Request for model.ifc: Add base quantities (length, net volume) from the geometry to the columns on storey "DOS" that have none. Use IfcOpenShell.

First a look at what the model holds.

```python
import ifcopenshell
import ifcopenshell.util.element
import ifcopenshell.util.unit

model = ifcopenshell.open("model.ifc")
print(model.schema)
for unit_type in ("LENGTHUNIT", "AREAUNIT", "VOLUMEUNIT"):
    print(unit_type, ifcopenshell.util.unit.calculate_unit_scale(model, unit_type))
storey = next(s for s in model.by_type("IfcBuildingStorey") if s.Name == "DOS")
columns = [e for e in ifcopenshell.util.element.get_decomposition(storey) if e.is_a("IfcColumn")]
for e in sorted(columns, key=lambda e: e.id()):
    print(e.id(), e.is_a(), e.Name, list(ifcopenshell.util.element.get_psets(e, qtos_only=True)), sep=" | ")
```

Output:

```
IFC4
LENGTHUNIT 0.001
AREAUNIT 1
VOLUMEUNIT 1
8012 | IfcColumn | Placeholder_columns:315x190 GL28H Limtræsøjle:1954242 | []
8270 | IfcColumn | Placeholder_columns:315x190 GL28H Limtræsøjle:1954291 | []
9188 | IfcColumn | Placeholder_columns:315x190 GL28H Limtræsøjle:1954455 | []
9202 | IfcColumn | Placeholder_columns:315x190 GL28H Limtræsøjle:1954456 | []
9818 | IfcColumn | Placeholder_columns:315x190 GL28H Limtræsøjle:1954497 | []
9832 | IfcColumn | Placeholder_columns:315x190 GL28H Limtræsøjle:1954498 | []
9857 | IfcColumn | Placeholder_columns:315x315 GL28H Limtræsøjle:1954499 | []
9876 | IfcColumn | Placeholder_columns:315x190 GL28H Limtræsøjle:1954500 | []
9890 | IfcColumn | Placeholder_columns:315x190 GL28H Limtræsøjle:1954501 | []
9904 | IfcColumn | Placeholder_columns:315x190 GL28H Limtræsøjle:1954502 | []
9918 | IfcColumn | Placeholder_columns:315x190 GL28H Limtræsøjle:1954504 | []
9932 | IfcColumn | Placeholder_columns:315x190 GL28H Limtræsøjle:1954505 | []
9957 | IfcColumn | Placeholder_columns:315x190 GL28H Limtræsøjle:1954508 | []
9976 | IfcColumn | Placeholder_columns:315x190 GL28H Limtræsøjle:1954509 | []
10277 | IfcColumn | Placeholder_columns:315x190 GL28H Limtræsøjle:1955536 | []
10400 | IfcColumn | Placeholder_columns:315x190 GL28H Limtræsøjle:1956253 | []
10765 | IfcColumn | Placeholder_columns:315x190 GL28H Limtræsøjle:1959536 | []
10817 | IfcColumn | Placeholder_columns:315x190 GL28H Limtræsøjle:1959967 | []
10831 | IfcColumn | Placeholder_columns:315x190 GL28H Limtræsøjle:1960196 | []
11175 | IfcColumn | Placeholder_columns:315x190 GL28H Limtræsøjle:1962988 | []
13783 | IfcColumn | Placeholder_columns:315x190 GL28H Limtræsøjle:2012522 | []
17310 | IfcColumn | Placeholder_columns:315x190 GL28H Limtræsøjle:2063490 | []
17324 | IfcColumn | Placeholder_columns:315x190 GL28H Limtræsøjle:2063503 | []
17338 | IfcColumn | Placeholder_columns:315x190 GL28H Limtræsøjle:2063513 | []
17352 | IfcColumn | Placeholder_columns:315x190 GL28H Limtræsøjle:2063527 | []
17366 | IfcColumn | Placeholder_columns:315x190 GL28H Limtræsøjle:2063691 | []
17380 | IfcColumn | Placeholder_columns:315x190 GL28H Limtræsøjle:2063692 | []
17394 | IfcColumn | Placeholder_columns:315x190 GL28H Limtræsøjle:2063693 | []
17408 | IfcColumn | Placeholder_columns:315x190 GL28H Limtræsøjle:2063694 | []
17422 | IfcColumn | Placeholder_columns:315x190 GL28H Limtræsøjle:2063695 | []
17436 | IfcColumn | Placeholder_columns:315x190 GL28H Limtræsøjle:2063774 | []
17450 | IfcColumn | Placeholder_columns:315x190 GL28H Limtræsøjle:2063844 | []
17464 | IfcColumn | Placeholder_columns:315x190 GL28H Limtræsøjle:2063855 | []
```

```python
import ifcopenshell
import ifcopenshell.api.pset
import ifcopenshell.geom
import ifcopenshell.util.element
import ifcopenshell.util.shape
import ifcopenshell.util.unit

model = ifcopenshell.open("model.ifc")
unit_scale = ifcopenshell.util.unit.calculate_unit_scale(model)
volume_scale = ifcopenshell.util.unit.calculate_unit_scale(model, "VOLUMEUNIT")
settings = ifcopenshell.geom.settings()

storey = next(s for s in model.by_type("IfcBuildingStorey") if s.Name == "DOS")
columns = [e for e in ifcopenshell.util.element.get_decomposition(storey) if e.is_a("IfcColumn")]

for e in sorted(columns, key=lambda e: e.id()):
    if ifcopenshell.util.element.get_psets(e, qtos_only=True, should_inherit=False):
        continue
    # Geometry comes back in metres, in the element's own axes.
    shape = ifcopenshell.geom.create_shape(settings, e)
    values = {
        "Length": ifcopenshell.util.shape.get_z(shape.geometry) / unit_scale,
        "NetVolume": ifcopenshell.util.shape.get_volume(shape.geometry) / volume_scale,
    }
    qto = ifcopenshell.api.pset.add_qto(model, product=e, name="Qto_ColumnBaseQuantities")
    ifcopenshell.api.pset.edit_qto(model, qto=qto, properties=values)
    print(e.id(), {k: round(v, 3) for k, v in values.items()})

model.write("model_v2.ifc")
```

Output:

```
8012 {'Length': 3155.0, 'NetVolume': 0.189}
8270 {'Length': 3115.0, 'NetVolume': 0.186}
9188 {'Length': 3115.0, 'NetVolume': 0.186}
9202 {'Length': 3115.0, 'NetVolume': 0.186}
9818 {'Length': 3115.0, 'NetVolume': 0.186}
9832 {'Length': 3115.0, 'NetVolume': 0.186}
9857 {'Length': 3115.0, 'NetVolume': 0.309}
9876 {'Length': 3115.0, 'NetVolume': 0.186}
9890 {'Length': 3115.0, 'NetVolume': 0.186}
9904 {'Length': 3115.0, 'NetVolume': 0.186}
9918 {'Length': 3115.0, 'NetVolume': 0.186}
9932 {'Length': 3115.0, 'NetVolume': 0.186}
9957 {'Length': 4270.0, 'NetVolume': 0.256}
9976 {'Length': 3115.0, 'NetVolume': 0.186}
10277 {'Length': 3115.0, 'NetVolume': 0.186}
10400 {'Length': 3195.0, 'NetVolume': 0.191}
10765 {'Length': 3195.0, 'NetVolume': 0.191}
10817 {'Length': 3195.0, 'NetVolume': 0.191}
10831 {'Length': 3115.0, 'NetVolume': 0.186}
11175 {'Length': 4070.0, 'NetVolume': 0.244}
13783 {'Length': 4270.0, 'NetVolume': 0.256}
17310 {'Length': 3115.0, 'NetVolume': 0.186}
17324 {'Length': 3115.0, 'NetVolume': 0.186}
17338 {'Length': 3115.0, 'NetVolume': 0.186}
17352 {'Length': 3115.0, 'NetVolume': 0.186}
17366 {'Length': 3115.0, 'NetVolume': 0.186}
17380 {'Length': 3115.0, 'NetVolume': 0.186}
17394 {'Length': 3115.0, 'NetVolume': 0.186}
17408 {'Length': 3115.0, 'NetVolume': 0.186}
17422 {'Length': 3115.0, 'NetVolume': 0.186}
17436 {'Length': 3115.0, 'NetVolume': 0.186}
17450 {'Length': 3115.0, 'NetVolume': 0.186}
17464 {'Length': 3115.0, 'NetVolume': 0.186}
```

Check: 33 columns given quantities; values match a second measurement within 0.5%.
